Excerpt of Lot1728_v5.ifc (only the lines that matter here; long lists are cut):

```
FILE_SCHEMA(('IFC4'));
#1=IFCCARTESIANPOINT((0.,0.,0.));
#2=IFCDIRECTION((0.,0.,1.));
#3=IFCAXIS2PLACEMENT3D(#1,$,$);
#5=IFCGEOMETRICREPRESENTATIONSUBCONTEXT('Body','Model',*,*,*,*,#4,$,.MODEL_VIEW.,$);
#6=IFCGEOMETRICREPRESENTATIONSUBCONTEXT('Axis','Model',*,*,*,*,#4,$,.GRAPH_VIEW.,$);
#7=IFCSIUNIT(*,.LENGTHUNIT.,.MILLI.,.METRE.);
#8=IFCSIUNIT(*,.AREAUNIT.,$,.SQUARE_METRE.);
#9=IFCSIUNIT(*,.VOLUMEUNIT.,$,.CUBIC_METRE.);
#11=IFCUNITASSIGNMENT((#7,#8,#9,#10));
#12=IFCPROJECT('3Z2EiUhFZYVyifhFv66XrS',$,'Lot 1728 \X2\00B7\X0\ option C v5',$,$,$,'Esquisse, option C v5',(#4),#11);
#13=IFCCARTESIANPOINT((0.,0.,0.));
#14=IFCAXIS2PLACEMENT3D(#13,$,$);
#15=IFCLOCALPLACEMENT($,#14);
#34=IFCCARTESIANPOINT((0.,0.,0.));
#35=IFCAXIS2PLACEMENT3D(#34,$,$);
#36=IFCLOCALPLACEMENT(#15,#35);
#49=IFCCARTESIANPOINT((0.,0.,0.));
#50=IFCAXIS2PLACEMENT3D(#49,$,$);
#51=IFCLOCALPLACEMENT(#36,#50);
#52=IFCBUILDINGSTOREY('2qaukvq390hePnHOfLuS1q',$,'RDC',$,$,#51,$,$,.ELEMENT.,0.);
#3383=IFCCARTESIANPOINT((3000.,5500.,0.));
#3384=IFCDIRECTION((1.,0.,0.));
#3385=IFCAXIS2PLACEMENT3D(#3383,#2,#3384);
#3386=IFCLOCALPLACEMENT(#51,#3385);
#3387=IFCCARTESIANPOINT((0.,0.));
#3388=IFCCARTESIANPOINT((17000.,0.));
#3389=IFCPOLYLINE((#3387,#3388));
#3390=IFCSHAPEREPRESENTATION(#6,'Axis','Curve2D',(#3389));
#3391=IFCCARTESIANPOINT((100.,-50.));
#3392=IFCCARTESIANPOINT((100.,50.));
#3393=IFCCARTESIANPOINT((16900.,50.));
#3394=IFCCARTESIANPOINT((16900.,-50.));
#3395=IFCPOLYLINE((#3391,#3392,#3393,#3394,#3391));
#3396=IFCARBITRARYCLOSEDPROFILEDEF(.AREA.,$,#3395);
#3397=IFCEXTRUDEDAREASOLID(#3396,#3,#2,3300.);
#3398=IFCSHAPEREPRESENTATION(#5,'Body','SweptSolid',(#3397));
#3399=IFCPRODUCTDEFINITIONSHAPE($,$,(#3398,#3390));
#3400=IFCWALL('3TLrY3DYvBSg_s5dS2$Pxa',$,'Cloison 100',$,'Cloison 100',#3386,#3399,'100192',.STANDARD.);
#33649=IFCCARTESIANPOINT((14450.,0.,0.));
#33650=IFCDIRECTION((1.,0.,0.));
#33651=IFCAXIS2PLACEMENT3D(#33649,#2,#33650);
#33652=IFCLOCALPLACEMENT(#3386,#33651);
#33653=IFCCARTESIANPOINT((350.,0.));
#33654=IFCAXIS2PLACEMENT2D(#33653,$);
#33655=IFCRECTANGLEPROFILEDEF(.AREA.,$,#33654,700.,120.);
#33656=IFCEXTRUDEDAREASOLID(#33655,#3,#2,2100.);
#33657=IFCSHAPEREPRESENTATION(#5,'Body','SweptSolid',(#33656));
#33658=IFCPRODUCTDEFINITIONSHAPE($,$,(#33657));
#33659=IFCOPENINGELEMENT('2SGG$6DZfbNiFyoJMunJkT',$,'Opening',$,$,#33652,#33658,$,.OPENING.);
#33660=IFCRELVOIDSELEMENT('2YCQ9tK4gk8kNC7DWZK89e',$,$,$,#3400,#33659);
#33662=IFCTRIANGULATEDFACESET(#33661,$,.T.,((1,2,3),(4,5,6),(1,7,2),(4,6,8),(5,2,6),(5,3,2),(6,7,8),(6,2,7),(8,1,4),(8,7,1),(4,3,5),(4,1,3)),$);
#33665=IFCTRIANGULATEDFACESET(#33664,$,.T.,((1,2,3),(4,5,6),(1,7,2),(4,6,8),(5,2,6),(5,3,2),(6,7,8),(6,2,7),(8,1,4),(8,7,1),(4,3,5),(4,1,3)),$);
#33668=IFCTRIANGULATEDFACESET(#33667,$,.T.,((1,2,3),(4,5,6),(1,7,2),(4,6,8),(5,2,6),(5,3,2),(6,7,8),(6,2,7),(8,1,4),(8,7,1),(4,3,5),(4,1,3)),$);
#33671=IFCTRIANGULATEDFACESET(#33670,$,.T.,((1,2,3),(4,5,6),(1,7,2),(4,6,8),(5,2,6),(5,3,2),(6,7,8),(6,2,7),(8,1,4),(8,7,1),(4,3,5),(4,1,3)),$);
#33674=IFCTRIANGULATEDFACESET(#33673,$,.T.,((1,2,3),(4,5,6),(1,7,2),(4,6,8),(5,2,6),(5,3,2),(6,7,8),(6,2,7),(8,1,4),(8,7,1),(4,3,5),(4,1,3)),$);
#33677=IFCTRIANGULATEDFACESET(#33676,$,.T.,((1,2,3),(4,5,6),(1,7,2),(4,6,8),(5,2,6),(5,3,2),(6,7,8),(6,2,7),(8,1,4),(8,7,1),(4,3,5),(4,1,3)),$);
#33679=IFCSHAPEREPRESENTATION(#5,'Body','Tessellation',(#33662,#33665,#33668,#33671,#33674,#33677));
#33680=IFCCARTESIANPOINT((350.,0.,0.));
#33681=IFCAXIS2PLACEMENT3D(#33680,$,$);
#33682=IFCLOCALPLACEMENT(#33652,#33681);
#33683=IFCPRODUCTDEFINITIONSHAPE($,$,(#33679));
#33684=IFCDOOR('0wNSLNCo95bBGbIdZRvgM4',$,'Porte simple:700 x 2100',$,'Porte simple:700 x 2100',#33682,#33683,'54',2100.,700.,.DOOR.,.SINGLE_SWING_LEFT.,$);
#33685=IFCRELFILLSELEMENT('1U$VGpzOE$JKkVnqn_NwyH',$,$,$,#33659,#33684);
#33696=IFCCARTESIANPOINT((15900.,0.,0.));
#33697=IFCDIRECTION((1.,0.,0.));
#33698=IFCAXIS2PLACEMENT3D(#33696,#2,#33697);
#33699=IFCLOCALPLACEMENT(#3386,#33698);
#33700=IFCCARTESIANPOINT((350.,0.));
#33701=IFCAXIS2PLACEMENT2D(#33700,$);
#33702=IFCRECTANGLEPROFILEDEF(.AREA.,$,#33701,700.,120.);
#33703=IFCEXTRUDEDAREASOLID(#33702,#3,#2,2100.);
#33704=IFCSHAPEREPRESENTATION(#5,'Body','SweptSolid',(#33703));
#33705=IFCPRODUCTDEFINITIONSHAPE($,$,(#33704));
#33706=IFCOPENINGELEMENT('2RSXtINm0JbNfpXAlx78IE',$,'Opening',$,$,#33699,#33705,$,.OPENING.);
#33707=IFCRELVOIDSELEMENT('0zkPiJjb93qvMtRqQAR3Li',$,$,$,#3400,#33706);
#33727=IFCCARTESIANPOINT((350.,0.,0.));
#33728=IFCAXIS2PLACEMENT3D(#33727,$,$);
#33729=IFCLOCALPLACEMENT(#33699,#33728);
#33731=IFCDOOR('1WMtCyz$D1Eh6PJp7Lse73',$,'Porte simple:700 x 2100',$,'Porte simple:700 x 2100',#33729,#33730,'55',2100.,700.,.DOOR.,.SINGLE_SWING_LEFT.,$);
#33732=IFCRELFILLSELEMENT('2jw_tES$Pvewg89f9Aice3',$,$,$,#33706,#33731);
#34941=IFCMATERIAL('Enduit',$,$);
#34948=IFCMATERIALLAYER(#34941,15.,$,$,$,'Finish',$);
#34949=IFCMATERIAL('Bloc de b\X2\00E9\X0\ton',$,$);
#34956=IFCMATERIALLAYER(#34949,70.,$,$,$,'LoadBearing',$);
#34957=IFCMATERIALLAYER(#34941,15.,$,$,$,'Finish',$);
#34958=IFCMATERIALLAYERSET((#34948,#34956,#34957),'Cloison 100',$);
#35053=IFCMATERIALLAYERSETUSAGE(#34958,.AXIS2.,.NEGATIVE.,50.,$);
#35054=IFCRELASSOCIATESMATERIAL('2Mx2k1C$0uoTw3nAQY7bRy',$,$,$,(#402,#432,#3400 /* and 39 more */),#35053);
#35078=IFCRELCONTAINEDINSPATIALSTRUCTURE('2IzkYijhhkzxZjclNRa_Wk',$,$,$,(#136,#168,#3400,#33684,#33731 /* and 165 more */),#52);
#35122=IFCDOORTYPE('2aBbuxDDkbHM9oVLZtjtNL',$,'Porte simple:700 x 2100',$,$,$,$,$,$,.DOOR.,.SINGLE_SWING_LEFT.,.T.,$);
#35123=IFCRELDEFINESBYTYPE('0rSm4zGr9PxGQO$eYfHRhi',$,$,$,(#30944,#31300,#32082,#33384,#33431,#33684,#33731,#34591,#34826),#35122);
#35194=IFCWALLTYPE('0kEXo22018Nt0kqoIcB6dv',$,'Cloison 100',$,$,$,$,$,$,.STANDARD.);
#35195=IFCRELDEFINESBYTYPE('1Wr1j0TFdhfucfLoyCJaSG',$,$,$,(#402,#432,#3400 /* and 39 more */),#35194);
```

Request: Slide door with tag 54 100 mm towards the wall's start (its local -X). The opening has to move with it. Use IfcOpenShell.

```python
import ifcopenshell
import ifcopenshell.api.geometry
import ifcopenshell.util.placement
import ifcopenshell.util.unit

model = ifcopenshell.open("Lot1728_v5.ifc")
unit_scale = ifcopenshell.util.unit.calculate_unit_scale(model)

door = model.by_guid("0wNSLNCo95bBGbIdZRvgM4")
opening = door.FillsVoids[0].RelatingOpeningElement
wall = opening.VoidsElements[0].RelatingBuildingElement

wall_matrix = ifcopenshell.util.placement.get_local_placement(wall.ObjectPlacement)
shift = wall_matrix[:3, 0] * -0.1 / unit_scale
before = ifcopenshell.util.placement.get_local_placement(door.ObjectPlacement)[:3, 3].copy()

# The door is placed relative to its opening, so it follows when the opening moves.
matrix = ifcopenshell.util.placement.get_local_placement(opening.ObjectPlacement)
matrix[:3, 3] += shift
ifcopenshell.api.geometry.edit_object_placement(
    model, product=opening, matrix=matrix, is_si=False, should_transform_children=True
)

after = ifcopenshell.util.placement.get_local_placement(door.ObjectPlacement)[:3, 3]
print("door moved by", (after - before).round(3) + 0.0)

model.write("Lot1728_v5-out.ifc")
```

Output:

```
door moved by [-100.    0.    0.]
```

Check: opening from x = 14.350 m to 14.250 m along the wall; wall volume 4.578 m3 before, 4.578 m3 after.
